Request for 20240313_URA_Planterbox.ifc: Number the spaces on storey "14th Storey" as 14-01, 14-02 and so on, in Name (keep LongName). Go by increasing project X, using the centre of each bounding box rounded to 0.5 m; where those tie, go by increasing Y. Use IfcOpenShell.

First a look at what the model holds.

```python
import ifcopenshell
import ifcopenshell.util.element
import ifcopenshell.util.placement

model = ifcopenshell.open("20240313_URA_Planterbox.ifc")
print(model.schema)
storey = next(s for s in model.by_type("IfcBuildingStorey") if s.Name == "14th Storey")
spaces = [e for e in ifcopenshell.util.element.get_decomposition(storey) if e.is_a("IfcSpace")]
for e in sorted(spaces, key=lambda e: e.id()):
    origin = ifcopenshell.util.placement.get_local_placement(e.ObjectPlacement)[:3, 3]
    print(e.id(), e.Name, e.LongName, origin.round(2) + 0.0, sep=" | ")
```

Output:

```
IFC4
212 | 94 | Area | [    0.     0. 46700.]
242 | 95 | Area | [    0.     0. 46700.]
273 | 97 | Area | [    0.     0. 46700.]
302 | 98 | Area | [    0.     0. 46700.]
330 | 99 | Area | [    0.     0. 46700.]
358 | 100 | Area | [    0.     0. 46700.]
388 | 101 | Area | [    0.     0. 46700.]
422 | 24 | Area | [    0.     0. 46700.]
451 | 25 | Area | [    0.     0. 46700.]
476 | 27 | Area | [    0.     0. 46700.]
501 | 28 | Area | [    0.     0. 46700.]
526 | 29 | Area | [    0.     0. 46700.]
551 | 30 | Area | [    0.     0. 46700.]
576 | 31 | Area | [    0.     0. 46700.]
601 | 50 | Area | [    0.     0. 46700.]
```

```python
import ifcopenshell
import ifcopenshell.geom
import ifcopenshell.util.element
import ifcopenshell.util.shape

model = ifcopenshell.open("20240313_URA_Planterbox.ifc")
settings = ifcopenshell.geom.settings()
settings.set("use-world-coords", True)


def centre(element):
    shape = ifcopenshell.geom.create_shape(settings, element)
    return ifcopenshell.util.shape.get_bbox_centroid(shape.geometry)


storey = next(s for s in model.by_type("IfcBuildingStorey") if s.Name == "14th Storey")
spaces = [e for e in ifcopenshell.util.element.get_decomposition(storey) if e.is_a("IfcSpace")]

# Insertion points can sit at a corner or the storey origin, so sort by the geometry (in metres).
centres = {e: centre(e) for e in spaces}
spaces.sort(key=lambda e: (round(centres[e][0] / 0.5), centres[e][1]))

for i, e in enumerate(spaces, start=1):
    number = f"14-{i:02d}"
    e.Name = number
    print(e.id(), number)

model.write("20240313_URA_Planterbox_edited.ifc")
```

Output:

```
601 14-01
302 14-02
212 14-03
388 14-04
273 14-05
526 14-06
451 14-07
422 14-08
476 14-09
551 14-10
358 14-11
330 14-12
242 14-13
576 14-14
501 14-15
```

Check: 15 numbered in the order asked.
